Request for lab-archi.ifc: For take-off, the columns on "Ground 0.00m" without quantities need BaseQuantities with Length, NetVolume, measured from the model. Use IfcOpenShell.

First a look at what the model holds.

```python
import ifcopenshell
import ifcopenshell.util.element
import ifcopenshell.util.unit

model = ifcopenshell.open("lab-archi.ifc")
print(model.schema)
for unit_type in ("LENGTHUNIT", "AREAUNIT", "VOLUMEUNIT"):
    print(unit_type, ifcopenshell.util.unit.calculate_unit_scale(model, unit_type))
storey = next(s for s in model.by_type("IfcBuildingStorey") if s.Name == "Ground 0.00m")
columns = [e for e in ifcopenshell.util.element.get_decomposition(storey) if e.is_a("IfcColumn")]
for e in sorted(columns, key=lambda e: e.id()):
    print(e.id(), e.is_a(), e.Name, list(ifcopenshell.util.element.get_psets(e, qtos_only=True)), sep=" | ")
```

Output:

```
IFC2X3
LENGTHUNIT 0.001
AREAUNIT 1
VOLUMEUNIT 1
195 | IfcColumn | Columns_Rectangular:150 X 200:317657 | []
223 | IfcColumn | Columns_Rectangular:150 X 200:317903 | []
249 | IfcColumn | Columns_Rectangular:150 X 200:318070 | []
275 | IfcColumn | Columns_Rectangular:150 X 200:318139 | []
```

```python
import ifcopenshell
import ifcopenshell.api.pset
import ifcopenshell.geom
import ifcopenshell.util.element
import ifcopenshell.util.shape
import ifcopenshell.util.unit

model = ifcopenshell.open("lab-archi.ifc")
unit_scale = ifcopenshell.util.unit.calculate_unit_scale(model)
volume_scale = ifcopenshell.util.unit.calculate_unit_scale(model, "VOLUMEUNIT")
settings = ifcopenshell.geom.settings()

storey = next(s for s in model.by_type("IfcBuildingStorey") if s.Name == "Ground 0.00m")
columns = [e for e in ifcopenshell.util.element.get_decomposition(storey) if e.is_a("IfcColumn")]

for e in sorted(columns, key=lambda e: e.id()):
    if ifcopenshell.util.element.get_psets(e, qtos_only=True, should_inherit=False):
        continue
    # Geometry comes back in metres, in the element's own axes.
    shape = ifcopenshell.geom.create_shape(settings, e)
    values = {
        "Length": ifcopenshell.util.shape.get_z(shape.geometry) / unit_scale,
        "NetVolume": ifcopenshell.util.shape.get_volume(shape.geometry) / volume_scale,
    }
    qto = ifcopenshell.api.pset.add_qto(model, product=e, name="BaseQuantities")
    ifcopenshell.api.pset.edit_qto(model, qto=qto, properties=values)
    print(e.id(), {k: round(v, 3) for k, v in values.items()})

model.write("lab-archi-out.ifc")
```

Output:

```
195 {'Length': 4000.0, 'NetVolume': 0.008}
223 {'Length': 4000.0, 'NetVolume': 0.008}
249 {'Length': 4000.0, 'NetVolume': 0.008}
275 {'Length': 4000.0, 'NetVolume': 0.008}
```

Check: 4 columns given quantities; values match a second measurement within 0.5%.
